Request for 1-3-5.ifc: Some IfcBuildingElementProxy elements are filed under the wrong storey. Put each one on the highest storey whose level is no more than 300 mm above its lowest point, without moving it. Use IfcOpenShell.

First a look at what the model holds.

```python
import ifcopenshell
import ifcopenshell.util.element
import ifcopenshell.util.placement

model = ifcopenshell.open("1-3-5.ifc")
print(model.schema)
for storey in model.by_type("IfcBuildingStorey"):
    level = ifcopenshell.util.placement.get_storey_elevation(storey)
    count = sum(e.is_a("IfcBuildingElementProxy") for e in ifcopenshell.util.element.get_contained(storey))
    print(storey.id(), storey.Name, round(level, 3), count, sep=" | ")
```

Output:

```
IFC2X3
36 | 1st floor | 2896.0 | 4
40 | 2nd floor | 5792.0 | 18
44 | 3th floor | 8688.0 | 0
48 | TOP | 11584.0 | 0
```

```python
import ifcopenshell
import ifcopenshell.api.spatial
import ifcopenshell.geom
import ifcopenshell.util.element
import ifcopenshell.util.placement
import ifcopenshell.util.shape
import ifcopenshell.util.unit

model = ifcopenshell.open("1-3-5.ifc")
unit_scale = ifcopenshell.util.unit.calculate_unit_scale(model)
settings = ifcopenshell.geom.settings()

levels = sorted(
    ((ifcopenshell.util.placement.get_storey_elevation(s) * unit_scale, s) for s in model.by_type("IfcBuildingStorey")),
    key=lambda pair: pair[0],
)

for e in model.by_type("IfcBuildingElementProxy"):
    current = e.ContainedInStructure[0].RelatingStructure if e.ContainedInStructure else None
    if current is None or not current.is_a("IfcBuildingStorey"):
        continue
    shape = ifcopenshell.geom.create_shape(settings, e)
    bottom = ifcopenshell.util.shape.get_shape_bottom_elevation(shape, shape.geometry)
    below = [s for level, s in levels if level <= bottom + 0.3]
    storey = below[-1] if below else levels[0][1]
    if storey != current:
        # assign_container keeps the world position.
        ifcopenshell.api.spatial.assign_container(model, products=[e], relating_structure=storey)
        print(e.id(), current.Name, "->", storey.Name)

model.write("1-3-5_updated.ifc")
```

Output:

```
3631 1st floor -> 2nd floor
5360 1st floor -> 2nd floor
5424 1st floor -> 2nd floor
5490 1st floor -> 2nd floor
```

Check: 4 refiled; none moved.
